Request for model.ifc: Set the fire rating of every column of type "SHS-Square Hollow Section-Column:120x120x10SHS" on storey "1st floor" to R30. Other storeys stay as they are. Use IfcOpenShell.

First a look at what the model holds.

```python
import ifcopenshell
import ifcopenshell.util.element

model = ifcopenshell.open("model.ifc")
print(model.schema)
storey = next(s for s in model.by_type("IfcBuildingStorey") if s.Name == "1st floor")
columns = [e for e in ifcopenshell.util.element.get_decomposition(storey) if e.is_a("IfcColumn")]
seen = {}
for e in columns:
    element_type = ifcopenshell.util.element.get_type(e)
    key = (element_type.Name if element_type != e and element_type else None, ifcopenshell.util.element.get_pset(e, "Pset_ColumnCommon", "FireRating"))
    seen[key] = seen.get(key, 0) + 1
for (name, value), count in sorted(seen.items(), key=str):
    print(count, "x", name, "|", value)
```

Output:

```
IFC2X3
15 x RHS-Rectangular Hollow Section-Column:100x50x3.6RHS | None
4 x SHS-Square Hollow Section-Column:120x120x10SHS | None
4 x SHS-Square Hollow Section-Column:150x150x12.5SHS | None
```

```python
import ifcopenshell
import ifcopenshell.api.pset
import ifcopenshell.util.element

model = ifcopenshell.open("model.ifc")

storey = next(s for s in model.by_type("IfcBuildingStorey") if s.Name == "1st floor")
columns = [e for e in ifcopenshell.util.element.get_decomposition(storey) if e.is_a("IfcColumn")]

count = 0
for e in columns:
    element_type = ifcopenshell.util.element.get_type(e)
    if element_type in (None, e) or element_type.Name != "SHS-Square Hollow Section-Column:120x120x10SHS":
        continue
    # add_pset returns the element's existing set when there is one.
    pset = ifcopenshell.api.pset.add_pset(model, product=e, name="Pset_ColumnCommon")
    ifcopenshell.api.pset.edit_pset(model, pset=pset, properties={"FireRating": "R30"})
    count += 1

print(count, "columns updated")

model.write("model_edited.ifc")
```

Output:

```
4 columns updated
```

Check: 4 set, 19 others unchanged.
